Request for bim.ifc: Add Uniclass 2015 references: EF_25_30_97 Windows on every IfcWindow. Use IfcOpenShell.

First a look at what the model holds.

```python
import ifcopenshell

model = ifcopenshell.open("bim.ifc")
print(model.schema)
print("classifications:", [c.Name for c in model.by_type("IfcClassification")])
for ifc_class in ("IfcDoor", "IfcRoof", "IfcStair", "IfcWall", "IfcWindow"):
    print(ifc_class, len(model.by_type(ifc_class)))
```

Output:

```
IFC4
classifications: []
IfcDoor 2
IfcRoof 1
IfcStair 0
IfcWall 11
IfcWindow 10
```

```python
import ifcopenshell
import ifcopenshell.api.classification

model = ifcopenshell.open("bim.ifc")

system = ifcopenshell.api.classification.add_classification(model, classification="Uniclass 2015")

codes = {
    "IfcWindow": ("EF_25_30_97", "Windows"),
}
for ifc_class, (code, name) in codes.items():
    products = model.by_type(ifc_class)
    ifcopenshell.api.classification.add_reference(
        model, products=products, classification=system, identification=code, name=name
    )
    print(code, len(products))

model.write("bim-out.ifc")
```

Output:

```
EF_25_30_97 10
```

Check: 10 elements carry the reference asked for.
